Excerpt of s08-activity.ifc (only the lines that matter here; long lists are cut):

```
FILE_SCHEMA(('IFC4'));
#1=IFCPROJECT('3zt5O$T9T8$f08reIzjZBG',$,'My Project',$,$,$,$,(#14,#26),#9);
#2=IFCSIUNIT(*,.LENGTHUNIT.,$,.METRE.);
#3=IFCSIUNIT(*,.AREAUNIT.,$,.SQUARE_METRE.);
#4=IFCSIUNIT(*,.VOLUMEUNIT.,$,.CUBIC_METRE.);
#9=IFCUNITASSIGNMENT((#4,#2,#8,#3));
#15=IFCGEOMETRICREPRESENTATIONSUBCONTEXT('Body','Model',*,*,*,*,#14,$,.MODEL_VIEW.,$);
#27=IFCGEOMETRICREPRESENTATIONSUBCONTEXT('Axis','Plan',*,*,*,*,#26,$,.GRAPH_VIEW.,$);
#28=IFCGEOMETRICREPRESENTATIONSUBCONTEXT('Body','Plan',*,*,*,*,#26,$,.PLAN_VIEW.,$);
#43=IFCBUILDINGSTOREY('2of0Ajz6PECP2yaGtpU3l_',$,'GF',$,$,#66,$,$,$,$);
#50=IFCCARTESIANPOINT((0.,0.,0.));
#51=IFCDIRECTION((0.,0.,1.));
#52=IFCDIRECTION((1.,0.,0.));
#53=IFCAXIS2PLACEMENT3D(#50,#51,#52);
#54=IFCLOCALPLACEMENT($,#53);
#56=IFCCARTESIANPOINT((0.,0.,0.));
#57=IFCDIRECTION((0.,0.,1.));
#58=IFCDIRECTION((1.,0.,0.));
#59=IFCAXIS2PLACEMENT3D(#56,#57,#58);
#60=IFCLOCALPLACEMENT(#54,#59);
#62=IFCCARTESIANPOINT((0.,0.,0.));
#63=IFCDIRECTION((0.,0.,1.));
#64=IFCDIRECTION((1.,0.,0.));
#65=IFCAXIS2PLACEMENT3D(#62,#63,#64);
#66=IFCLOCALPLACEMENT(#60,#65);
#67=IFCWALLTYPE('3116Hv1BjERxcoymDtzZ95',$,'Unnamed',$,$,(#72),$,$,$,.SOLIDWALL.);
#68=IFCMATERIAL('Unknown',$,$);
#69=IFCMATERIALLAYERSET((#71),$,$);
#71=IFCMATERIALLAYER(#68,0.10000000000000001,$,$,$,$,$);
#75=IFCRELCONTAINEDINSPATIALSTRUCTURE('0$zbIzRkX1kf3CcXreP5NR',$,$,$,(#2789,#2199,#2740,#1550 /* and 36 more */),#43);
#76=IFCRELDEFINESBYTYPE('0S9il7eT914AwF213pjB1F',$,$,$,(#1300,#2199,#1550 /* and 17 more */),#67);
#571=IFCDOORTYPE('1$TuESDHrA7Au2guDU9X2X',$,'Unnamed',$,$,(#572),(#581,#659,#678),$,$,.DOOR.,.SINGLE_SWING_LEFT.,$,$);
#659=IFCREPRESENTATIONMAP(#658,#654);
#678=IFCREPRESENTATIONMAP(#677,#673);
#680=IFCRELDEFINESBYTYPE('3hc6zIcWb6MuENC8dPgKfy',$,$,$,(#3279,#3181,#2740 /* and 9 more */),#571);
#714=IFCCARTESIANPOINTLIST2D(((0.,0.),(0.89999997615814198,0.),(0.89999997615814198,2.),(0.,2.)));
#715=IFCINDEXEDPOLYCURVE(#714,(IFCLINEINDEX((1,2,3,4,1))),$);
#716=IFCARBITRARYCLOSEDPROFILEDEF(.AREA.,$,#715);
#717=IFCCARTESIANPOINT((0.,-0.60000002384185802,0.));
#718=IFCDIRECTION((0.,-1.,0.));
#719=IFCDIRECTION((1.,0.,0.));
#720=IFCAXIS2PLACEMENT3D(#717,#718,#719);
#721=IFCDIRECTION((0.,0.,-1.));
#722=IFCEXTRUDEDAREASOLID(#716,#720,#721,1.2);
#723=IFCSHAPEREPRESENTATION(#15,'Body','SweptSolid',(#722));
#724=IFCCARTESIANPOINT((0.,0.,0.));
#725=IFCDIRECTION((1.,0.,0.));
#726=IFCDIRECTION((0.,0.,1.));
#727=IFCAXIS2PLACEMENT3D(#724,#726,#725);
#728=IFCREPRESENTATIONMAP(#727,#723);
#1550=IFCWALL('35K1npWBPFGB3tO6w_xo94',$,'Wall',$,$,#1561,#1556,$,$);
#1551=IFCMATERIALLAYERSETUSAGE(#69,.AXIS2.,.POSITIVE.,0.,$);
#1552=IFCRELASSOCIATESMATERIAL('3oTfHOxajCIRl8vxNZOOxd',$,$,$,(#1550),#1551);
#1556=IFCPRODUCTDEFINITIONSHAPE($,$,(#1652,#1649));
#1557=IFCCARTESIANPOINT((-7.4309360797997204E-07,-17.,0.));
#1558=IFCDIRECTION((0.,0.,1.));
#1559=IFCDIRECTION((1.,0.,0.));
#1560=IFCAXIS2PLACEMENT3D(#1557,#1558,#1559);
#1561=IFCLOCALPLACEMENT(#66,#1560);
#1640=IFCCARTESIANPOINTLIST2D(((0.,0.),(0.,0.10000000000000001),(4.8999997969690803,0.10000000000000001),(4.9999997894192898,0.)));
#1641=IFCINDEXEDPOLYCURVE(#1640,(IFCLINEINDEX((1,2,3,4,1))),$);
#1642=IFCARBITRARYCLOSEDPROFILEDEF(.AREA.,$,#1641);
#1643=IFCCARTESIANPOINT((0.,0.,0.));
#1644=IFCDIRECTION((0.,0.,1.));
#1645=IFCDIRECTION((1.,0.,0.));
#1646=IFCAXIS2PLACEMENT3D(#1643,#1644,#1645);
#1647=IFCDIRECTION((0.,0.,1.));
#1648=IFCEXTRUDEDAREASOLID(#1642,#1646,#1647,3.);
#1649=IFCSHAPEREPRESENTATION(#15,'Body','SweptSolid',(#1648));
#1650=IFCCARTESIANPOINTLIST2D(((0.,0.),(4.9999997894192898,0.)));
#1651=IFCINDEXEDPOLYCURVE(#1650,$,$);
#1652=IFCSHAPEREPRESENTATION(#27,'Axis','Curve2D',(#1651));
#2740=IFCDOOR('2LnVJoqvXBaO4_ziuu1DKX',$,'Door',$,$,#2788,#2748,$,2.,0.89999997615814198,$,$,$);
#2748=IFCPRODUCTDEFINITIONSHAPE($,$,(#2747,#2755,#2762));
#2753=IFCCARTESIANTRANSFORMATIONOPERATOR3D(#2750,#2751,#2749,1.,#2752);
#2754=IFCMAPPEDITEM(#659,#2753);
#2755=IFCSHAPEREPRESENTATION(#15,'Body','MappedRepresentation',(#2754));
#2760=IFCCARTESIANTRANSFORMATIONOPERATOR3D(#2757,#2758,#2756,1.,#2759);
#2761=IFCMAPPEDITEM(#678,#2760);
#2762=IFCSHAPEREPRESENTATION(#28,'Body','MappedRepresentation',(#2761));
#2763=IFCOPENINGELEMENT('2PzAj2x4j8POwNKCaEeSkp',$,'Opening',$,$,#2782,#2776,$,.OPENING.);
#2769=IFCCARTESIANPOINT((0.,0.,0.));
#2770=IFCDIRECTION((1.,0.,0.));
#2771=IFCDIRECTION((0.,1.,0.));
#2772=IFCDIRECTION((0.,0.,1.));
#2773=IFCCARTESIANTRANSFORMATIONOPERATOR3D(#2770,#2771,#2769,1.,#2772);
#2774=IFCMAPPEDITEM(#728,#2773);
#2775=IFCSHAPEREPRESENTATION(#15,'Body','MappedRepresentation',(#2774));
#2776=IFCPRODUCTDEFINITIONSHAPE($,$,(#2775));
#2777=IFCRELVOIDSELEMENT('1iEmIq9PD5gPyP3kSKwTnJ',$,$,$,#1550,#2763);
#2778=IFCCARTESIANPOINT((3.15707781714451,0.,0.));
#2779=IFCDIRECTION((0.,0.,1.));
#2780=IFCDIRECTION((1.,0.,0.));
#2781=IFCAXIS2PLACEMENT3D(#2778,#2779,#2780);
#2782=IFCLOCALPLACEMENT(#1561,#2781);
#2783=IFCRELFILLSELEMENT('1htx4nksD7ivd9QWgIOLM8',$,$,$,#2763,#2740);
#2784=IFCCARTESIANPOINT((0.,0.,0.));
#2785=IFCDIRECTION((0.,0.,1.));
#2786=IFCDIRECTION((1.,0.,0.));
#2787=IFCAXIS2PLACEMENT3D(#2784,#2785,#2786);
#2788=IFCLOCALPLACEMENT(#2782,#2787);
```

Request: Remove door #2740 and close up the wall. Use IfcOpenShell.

```python
import ifcopenshell
import ifcopenshell.api.feature
import ifcopenshell.api.root
import ifcopenshell.geom
import ifcopenshell.util.shape

model = ifcopenshell.open("s08-activity.ifc")
settings = ifcopenshell.geom.settings()


def volume(element):
    """Net volume in cubic metres, openings subtracted."""
    shape = ifcopenshell.geom.create_shape(settings, element)
    return ifcopenshell.util.shape.get_volume(shape.geometry)


door = model.by_guid("2LnVJoqvXBaO4_ziuu1DKX")
opening = door.FillsVoids[0].RelatingOpeningElement
wall = opening.VoidsElements[0].RelatingBuildingElement
before = volume(wall)

ifcopenshell.api.root.remove_product(model, product=door)
ifcopenshell.api.feature.remove_feature(model, feature=opening)

after = volume(wall)

print(f"wall volume {before:.3f} -> {after:.3f} m3")

model.write("s08-activity_edited.ifc")
```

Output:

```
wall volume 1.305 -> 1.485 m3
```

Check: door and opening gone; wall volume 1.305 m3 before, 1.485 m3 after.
